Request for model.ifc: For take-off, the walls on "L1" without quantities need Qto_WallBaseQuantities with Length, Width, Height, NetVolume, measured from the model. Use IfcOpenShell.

First a look at what the model holds.

```python
import ifcopenshell
import ifcopenshell.util.element
import ifcopenshell.util.unit

model = ifcopenshell.open("model.ifc")
print(model.schema)
for unit_type in ("LENGTHUNIT", "AREAUNIT", "VOLUMEUNIT"):
    print(unit_type, ifcopenshell.util.unit.calculate_unit_scale(model, unit_type))
storey = next(s for s in model.by_type("IfcBuildingStorey") if s.Name == "L1")
walls = [e for e in ifcopenshell.util.element.get_decomposition(storey) if e.is_a("IfcWall")]
for e in sorted(walls, key=lambda e: e.id()):
    print(e.id(), e.is_a(), e.Name, list(ifcopenshell.util.element.get_psets(e, qtos_only=True)), sep=" | ")
```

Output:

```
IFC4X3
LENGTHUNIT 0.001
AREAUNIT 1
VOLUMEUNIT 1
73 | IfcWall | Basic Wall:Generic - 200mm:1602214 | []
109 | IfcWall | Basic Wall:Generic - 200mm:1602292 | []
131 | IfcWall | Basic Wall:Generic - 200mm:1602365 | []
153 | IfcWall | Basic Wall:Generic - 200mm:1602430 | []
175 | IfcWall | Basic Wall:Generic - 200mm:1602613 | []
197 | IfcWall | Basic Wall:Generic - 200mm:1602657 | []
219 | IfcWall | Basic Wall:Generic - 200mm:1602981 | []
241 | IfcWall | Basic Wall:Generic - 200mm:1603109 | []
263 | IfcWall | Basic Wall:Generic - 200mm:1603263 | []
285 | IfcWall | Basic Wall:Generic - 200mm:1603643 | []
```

```python
import ifcopenshell
import ifcopenshell.api.pset
import ifcopenshell.geom
import ifcopenshell.util.element
import ifcopenshell.util.shape
import ifcopenshell.util.unit

model = ifcopenshell.open("model.ifc")
unit_scale = ifcopenshell.util.unit.calculate_unit_scale(model)
volume_scale = ifcopenshell.util.unit.calculate_unit_scale(model, "VOLUMEUNIT")
settings = ifcopenshell.geom.settings()

storey = next(s for s in model.by_type("IfcBuildingStorey") if s.Name == "L1")
walls = [e for e in ifcopenshell.util.element.get_decomposition(storey) if e.is_a("IfcWall")]

for e in sorted(walls, key=lambda e: e.id()):
    if ifcopenshell.util.element.get_psets(e, qtos_only=True, should_inherit=False):
        continue
    # Geometry comes back in metres, in the element's own axes.
    shape = ifcopenshell.geom.create_shape(settings, e)
    values = {
        "Length": ifcopenshell.util.shape.get_x(shape.geometry) / unit_scale,
        "Width": ifcopenshell.util.shape.get_y(shape.geometry) / unit_scale,
        "Height": ifcopenshell.util.shape.get_z(shape.geometry) / unit_scale,
        "NetVolume": ifcopenshell.util.shape.get_volume(shape.geometry) / volume_scale,
    }
    qto = ifcopenshell.api.pset.add_qto(model, product=e, name="Qto_WallBaseQuantities")
    ifcopenshell.api.pset.edit_qto(model, qto=qto, properties=values)
    print(e.id(), {k: round(v, 3) for k, v in values.items()})

model.write("model-out.ifc")
```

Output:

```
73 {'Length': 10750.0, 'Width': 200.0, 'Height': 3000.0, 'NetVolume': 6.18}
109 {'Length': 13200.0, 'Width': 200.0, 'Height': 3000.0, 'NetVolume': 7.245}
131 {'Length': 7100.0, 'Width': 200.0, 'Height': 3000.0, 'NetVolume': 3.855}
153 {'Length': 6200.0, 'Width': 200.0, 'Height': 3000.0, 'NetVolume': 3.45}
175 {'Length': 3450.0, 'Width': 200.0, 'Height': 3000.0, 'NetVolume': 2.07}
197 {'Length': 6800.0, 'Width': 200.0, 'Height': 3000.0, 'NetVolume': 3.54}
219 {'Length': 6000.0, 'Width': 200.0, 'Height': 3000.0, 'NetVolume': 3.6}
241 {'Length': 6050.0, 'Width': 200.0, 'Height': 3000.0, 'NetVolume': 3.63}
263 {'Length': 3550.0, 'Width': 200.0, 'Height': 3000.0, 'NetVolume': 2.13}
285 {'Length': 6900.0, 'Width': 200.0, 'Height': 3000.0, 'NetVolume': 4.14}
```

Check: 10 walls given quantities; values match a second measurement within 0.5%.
